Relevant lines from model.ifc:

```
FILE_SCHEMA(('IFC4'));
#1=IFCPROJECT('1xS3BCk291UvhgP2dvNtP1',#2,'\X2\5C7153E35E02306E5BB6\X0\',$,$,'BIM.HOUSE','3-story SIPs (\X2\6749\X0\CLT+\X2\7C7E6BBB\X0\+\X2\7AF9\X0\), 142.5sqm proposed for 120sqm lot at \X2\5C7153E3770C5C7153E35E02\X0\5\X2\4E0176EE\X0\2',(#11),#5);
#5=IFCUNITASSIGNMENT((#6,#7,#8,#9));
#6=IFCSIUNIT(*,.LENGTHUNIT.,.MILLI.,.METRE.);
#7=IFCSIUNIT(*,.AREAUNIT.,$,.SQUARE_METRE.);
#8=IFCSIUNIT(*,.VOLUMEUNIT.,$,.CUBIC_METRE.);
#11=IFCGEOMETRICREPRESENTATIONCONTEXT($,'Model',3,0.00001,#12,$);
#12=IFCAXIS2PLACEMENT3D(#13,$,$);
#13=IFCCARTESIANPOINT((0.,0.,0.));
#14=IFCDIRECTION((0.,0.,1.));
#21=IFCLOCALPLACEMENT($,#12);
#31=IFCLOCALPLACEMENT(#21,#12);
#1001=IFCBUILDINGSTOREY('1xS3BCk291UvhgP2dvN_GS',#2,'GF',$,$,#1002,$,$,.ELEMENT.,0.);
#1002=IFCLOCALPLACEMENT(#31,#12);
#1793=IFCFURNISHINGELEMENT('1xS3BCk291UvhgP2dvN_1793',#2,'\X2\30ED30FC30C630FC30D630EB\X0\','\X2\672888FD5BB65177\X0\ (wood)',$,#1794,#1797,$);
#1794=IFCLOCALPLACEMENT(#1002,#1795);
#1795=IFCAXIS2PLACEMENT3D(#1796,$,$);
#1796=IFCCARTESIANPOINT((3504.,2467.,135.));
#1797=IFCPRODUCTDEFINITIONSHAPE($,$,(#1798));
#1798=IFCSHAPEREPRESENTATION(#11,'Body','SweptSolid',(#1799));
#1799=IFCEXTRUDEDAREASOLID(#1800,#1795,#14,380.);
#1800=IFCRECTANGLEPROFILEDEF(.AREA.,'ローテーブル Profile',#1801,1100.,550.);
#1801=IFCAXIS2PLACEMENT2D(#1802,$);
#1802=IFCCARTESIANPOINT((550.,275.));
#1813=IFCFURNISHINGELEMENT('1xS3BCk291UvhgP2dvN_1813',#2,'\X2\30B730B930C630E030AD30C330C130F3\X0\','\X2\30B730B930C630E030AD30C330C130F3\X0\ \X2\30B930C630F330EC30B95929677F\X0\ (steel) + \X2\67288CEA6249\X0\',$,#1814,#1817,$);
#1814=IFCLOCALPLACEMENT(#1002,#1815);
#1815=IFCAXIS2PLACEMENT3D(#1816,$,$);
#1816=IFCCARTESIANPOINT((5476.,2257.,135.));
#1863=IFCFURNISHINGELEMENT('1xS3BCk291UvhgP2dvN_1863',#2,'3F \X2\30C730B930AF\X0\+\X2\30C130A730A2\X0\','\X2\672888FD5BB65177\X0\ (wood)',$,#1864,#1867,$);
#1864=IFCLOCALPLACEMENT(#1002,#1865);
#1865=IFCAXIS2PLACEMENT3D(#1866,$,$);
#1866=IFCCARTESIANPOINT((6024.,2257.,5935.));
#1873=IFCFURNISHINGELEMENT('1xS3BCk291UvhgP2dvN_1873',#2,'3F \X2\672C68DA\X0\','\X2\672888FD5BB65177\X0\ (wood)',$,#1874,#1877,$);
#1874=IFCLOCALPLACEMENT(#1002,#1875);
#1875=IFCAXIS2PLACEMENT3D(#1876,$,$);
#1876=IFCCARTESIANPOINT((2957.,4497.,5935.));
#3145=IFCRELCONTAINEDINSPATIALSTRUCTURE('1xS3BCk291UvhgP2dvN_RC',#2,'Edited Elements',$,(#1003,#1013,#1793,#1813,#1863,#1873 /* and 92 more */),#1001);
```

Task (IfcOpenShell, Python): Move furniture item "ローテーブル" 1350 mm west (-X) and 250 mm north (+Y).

```python
import ifcopenshell
import ifcopenshell.api.geometry
import ifcopenshell.util.placement
import ifcopenshell.util.unit

model = ifcopenshell.open("model.ifc")
unit_scale = ifcopenshell.util.unit.calculate_unit_scale(model)

item = model.by_id(1793)
matrix = ifcopenshell.util.placement.get_local_placement(item.ObjectPlacement)
matrix[0, 3] -= 1.35 / unit_scale
matrix[1, 3] += 0.25 / unit_scale
ifcopenshell.api.geometry.edit_object_placement(model, product=item, matrix=matrix, is_si=False)

print(ifcopenshell.util.placement.get_local_placement(item.ObjectPlacement).round(3) + 0.0)

model.write("model_updated.ifc")
```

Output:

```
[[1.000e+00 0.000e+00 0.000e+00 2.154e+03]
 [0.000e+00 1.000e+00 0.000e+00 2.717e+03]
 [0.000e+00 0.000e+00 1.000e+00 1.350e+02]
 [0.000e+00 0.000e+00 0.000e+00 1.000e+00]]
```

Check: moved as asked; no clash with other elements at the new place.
